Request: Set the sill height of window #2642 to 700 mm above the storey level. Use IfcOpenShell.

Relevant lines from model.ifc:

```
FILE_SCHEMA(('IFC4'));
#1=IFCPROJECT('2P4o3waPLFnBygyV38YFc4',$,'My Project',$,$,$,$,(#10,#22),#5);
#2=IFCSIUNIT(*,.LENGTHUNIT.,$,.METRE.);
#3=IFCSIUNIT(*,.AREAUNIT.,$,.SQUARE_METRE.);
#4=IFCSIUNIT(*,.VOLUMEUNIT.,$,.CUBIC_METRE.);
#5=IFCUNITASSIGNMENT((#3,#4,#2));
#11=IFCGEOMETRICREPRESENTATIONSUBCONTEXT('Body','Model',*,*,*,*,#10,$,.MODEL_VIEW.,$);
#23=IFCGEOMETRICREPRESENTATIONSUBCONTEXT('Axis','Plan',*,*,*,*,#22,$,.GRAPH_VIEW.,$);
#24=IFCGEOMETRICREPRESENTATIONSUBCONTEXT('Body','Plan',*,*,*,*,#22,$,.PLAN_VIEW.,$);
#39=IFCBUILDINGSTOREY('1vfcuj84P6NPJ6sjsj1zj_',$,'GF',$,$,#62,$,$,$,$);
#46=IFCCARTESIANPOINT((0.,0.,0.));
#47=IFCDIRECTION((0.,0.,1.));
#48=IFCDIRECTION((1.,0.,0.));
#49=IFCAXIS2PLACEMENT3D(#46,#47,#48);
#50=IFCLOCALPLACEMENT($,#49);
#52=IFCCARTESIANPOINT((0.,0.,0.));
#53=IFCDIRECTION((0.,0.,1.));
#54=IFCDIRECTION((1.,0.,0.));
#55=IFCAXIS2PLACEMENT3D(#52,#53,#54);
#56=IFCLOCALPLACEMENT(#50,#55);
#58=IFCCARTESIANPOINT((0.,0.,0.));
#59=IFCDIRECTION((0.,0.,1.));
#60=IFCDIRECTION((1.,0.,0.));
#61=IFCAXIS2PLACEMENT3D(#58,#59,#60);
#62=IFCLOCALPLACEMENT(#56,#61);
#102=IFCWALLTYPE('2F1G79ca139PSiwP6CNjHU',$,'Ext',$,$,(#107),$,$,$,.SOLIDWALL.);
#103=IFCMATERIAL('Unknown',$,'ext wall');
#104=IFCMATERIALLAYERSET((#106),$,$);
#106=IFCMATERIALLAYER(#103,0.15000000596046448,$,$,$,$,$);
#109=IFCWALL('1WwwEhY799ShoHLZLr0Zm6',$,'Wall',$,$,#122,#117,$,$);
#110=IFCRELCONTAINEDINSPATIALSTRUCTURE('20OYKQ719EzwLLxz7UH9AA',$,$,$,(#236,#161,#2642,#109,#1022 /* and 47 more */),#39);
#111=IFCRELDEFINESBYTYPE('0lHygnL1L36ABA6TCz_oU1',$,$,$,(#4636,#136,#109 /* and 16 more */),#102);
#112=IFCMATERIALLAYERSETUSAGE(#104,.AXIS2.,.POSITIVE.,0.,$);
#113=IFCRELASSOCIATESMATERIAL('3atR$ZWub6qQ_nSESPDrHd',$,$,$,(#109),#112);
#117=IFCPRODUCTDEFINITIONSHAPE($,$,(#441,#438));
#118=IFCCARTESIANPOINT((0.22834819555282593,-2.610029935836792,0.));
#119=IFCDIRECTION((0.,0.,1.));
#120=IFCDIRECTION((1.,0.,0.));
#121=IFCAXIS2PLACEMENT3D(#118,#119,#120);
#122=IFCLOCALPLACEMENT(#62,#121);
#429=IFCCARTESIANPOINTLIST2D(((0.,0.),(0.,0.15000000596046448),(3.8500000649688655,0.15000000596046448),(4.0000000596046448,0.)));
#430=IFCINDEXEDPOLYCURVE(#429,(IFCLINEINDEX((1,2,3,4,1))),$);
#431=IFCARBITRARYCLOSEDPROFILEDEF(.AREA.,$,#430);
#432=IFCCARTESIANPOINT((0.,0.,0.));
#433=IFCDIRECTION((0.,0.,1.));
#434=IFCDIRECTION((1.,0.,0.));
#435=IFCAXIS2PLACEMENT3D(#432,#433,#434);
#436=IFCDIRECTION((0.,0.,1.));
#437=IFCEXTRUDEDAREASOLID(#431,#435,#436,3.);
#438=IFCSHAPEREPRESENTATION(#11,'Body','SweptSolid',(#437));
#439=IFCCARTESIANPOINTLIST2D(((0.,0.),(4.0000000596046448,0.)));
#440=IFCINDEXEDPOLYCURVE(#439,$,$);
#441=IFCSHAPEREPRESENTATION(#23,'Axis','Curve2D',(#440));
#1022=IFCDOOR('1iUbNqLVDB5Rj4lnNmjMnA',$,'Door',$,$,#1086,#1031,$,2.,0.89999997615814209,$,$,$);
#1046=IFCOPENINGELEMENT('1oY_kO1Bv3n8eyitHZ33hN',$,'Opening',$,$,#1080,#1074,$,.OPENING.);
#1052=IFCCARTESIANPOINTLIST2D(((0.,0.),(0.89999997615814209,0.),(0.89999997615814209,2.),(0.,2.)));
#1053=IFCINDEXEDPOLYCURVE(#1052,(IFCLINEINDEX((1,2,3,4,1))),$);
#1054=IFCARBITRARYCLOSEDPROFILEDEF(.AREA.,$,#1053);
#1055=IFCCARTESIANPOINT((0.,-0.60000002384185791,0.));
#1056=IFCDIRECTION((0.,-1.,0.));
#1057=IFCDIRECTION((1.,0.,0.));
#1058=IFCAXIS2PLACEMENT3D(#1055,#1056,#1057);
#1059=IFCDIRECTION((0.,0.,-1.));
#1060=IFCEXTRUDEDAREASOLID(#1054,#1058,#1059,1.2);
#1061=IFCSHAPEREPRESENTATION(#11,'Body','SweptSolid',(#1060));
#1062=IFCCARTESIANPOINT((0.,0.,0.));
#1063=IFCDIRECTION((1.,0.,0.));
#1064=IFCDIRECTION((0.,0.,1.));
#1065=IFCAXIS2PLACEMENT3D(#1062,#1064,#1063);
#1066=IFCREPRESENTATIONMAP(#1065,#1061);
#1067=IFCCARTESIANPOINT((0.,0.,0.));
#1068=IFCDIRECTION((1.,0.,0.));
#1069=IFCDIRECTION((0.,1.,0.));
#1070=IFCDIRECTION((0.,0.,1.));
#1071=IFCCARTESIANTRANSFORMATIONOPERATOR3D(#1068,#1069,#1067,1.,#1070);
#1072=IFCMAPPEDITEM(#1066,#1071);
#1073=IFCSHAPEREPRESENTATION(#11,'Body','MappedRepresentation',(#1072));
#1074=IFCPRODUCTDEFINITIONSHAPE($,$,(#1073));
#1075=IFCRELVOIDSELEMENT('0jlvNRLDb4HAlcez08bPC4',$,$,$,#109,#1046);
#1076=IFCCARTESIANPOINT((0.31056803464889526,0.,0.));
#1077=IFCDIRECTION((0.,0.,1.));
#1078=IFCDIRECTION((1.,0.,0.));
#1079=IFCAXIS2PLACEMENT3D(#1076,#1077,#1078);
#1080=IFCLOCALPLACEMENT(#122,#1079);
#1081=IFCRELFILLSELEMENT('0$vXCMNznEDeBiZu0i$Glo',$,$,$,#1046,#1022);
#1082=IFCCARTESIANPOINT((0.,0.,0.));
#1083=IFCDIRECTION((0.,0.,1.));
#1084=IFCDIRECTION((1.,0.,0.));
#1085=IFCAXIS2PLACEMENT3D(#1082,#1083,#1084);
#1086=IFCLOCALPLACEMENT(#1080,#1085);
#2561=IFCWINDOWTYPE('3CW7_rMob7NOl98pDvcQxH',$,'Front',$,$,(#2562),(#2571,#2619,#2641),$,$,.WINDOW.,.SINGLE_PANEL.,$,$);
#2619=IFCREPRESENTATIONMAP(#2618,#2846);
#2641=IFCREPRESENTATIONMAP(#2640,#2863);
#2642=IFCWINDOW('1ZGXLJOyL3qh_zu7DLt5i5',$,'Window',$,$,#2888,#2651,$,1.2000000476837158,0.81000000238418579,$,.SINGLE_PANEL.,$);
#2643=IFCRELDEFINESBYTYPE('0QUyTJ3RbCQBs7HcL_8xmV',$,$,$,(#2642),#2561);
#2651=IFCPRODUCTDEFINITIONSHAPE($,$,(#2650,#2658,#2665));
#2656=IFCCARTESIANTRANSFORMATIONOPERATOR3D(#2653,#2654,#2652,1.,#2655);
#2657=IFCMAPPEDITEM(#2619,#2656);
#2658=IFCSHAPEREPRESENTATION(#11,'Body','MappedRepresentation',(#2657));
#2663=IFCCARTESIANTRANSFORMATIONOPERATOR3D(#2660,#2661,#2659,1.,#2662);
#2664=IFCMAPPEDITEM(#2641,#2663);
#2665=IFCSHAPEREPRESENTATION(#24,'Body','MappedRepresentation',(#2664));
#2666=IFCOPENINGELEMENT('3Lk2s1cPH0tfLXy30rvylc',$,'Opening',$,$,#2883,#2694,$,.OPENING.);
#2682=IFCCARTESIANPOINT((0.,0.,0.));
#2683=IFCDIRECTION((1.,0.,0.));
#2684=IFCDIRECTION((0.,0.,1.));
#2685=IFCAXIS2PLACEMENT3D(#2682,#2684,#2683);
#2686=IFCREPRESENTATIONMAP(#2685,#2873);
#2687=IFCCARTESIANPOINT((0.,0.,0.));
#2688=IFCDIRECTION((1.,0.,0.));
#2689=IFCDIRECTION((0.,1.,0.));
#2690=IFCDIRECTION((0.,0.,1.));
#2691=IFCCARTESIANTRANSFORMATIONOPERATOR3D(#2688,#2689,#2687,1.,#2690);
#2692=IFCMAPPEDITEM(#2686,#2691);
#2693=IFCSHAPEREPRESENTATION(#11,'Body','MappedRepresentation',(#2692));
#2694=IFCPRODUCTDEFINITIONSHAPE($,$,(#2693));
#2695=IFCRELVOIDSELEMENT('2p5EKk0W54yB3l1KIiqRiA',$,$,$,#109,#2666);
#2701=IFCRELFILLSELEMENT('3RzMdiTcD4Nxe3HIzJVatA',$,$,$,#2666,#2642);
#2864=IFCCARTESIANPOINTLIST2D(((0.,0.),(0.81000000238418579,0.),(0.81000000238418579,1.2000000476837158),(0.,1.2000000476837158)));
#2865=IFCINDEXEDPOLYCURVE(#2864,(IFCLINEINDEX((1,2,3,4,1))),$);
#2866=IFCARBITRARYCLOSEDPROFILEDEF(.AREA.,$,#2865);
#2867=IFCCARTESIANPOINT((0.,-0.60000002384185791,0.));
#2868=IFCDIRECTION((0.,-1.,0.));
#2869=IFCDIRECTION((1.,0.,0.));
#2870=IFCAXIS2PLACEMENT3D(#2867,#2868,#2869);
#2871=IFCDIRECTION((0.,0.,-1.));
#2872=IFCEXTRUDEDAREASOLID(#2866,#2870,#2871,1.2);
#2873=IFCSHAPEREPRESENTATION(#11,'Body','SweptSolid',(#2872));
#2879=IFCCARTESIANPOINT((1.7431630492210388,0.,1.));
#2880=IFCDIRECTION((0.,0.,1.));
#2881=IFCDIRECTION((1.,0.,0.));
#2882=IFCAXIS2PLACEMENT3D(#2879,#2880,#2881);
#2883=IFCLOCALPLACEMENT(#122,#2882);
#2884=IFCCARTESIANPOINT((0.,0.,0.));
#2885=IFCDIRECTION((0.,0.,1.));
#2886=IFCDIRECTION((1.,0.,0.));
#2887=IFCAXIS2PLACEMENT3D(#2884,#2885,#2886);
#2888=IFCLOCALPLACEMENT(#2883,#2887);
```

```python
import numpy as np
import ifcopenshell
import ifcopenshell.api.geometry
import ifcopenshell.geom
import ifcopenshell.util.element
import ifcopenshell.util.placement
import ifcopenshell.util.shape
import ifcopenshell.util.unit

model = ifcopenshell.open("model.ifc")
unit_scale = ifcopenshell.util.unit.calculate_unit_scale(model)

window = model.by_guid("1ZGXLJOyL3qh_zu7DLt5i5")
opening = window.FillsVoids[0].RelatingOpeningElement
storey = ifcopenshell.util.element.get_container(window, ifc_class="IfcBuildingStorey")
level = ifcopenshell.util.placement.get_local_placement(storey.ObjectPlacement)[2, 3]

# The opening's origin need not be at the sill, so measure its lowest point.
shape = ifcopenshell.geom.create_shape(ifcopenshell.geom.settings(), opening)
bottom = ifcopenshell.util.shape.get_shape_bottom_elevation(shape, shape.geometry) / unit_scale
dz = level + 0.7 / unit_scale - bottom

shift = np.array([0.0, 0.0, dz])
# The window is placed relative to its opening, so it follows when the opening moves.
matrix = ifcopenshell.util.placement.get_local_placement(opening.ObjectPlacement)
matrix[:3, 3] += shift
ifcopenshell.api.geometry.edit_object_placement(
    model, product=opening, matrix=matrix, is_si=False, should_transform_children=True
)

print(f"moved by {dz * unit_scale:+.3f} m")

model.write("model_edited.ifc")
```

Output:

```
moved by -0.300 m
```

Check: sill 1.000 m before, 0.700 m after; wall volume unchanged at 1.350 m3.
